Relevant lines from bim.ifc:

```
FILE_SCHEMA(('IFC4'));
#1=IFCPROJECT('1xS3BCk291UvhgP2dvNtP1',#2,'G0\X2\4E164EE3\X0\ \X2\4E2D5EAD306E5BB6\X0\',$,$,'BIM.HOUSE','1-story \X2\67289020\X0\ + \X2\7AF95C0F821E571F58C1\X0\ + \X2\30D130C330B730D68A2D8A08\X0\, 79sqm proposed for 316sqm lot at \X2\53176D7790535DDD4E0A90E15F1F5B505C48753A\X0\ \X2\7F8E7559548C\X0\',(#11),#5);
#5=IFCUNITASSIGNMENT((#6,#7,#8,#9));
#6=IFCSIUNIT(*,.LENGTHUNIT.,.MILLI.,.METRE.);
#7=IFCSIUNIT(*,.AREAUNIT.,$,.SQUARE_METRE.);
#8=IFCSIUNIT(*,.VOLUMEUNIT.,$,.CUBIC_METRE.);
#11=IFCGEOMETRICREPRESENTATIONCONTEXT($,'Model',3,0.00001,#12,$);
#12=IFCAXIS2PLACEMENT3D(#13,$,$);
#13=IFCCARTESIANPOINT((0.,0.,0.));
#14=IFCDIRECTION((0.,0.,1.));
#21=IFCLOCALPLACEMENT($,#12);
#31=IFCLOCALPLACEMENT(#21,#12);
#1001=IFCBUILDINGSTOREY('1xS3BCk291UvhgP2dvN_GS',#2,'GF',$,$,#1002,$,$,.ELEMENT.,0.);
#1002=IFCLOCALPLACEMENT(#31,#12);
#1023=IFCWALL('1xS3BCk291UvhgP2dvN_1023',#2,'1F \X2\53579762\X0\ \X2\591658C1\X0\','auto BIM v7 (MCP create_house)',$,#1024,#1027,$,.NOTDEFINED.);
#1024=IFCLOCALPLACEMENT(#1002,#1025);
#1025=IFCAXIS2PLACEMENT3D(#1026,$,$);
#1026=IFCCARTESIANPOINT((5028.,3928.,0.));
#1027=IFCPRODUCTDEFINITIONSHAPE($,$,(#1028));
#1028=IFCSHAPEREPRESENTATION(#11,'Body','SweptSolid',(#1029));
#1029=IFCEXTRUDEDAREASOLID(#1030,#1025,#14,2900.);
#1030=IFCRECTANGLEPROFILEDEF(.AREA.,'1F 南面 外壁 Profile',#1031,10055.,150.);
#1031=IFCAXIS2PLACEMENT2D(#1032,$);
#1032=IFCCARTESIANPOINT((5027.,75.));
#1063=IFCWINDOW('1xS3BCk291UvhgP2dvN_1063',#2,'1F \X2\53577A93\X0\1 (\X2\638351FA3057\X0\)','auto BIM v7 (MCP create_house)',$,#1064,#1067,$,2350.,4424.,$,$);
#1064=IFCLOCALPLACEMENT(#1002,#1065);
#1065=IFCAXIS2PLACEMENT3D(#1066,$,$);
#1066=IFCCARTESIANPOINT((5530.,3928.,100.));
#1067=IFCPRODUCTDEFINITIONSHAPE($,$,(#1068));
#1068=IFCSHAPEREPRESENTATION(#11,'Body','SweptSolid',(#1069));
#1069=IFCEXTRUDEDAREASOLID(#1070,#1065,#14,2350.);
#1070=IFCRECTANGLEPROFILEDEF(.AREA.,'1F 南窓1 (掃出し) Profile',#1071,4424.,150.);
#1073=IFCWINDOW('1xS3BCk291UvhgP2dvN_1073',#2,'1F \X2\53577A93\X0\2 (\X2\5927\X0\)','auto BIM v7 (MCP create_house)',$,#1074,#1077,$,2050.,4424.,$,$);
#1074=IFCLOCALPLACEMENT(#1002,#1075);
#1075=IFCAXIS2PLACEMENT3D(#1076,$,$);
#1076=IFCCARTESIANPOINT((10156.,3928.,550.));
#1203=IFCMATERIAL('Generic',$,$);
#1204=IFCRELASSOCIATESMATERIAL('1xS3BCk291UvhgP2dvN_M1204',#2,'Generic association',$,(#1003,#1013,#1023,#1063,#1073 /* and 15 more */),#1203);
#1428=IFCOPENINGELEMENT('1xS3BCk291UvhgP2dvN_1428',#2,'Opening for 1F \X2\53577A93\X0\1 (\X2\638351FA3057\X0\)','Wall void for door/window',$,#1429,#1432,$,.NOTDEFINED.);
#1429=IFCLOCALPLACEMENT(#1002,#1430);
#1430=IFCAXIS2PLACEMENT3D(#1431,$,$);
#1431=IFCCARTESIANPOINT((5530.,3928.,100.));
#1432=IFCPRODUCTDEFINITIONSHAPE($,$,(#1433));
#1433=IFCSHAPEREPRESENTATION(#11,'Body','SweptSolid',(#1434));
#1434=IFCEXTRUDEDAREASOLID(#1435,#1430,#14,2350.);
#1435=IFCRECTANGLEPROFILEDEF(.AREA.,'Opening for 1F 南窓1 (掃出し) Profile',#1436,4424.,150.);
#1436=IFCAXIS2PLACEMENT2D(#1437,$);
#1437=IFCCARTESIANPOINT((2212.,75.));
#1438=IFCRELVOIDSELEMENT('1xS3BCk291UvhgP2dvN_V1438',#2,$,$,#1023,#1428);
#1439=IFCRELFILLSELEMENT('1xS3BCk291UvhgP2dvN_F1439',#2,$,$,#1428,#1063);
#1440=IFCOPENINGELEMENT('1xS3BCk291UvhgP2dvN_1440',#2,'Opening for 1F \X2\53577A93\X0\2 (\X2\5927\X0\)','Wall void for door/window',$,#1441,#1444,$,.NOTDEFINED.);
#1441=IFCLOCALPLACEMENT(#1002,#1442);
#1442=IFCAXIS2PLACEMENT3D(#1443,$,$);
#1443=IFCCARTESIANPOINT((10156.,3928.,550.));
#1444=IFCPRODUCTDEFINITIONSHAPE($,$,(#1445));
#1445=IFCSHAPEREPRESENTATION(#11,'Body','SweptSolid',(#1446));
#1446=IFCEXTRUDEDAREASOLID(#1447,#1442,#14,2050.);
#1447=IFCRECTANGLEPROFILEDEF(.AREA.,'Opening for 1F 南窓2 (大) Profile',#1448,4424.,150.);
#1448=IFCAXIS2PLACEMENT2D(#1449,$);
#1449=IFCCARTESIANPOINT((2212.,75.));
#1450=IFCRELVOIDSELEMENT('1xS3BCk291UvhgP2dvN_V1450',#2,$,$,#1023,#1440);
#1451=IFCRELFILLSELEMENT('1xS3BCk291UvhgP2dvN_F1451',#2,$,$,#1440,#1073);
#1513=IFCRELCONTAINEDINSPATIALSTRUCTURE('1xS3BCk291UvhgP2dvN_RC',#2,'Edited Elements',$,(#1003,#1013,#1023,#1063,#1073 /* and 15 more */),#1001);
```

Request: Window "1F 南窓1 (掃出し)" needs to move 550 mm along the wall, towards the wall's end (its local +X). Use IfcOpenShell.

```python
import ifcopenshell
import ifcopenshell.api.geometry
import ifcopenshell.util.placement
import ifcopenshell.util.unit

model = ifcopenshell.open("bim.ifc")
unit_scale = ifcopenshell.util.unit.calculate_unit_scale(model)

window = model.by_guid("1xS3BCk291UvhgP2dvN_1063")
opening = window.FillsVoids[0].RelatingOpeningElement
wall = opening.VoidsElements[0].RelatingBuildingElement

wall_matrix = ifcopenshell.util.placement.get_local_placement(wall.ObjectPlacement)
shift = wall_matrix[:3, 0] * 0.55 / unit_scale
before = ifcopenshell.util.placement.get_local_placement(window.ObjectPlacement)[:3, 3].copy()

# The window is not placed relative to its opening, so move both.
for product in (opening, window):
    matrix = ifcopenshell.util.placement.get_local_placement(product.ObjectPlacement)
    matrix[:3, 3] += shift
    ifcopenshell.api.geometry.edit_object_placement(model, product=product, matrix=matrix, is_si=False)

after = ifcopenshell.util.placement.get_local_placement(window.ObjectPlacement)[:3, 3]
print("window moved by", (after - before).round(3) + 0.0)

model.write("bim_edited.ifc")
```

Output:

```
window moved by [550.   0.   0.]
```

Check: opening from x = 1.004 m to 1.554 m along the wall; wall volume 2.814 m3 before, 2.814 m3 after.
